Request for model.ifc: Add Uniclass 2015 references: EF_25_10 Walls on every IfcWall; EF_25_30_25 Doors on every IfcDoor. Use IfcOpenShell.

First a look at what the model holds.

```python
import ifcopenshell

model = ifcopenshell.open("model.ifc")
print(model.schema)
print("classifications:", [c.Name for c in model.by_type("IfcClassification")])
for ifc_class in ("IfcDoor", "IfcRoof", "IfcStair", "IfcWall", "IfcWindow"):
    print(ifc_class, len(model.by_type(ifc_class)))
```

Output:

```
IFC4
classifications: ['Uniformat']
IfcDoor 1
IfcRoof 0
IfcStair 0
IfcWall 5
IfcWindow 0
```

```python
import ifcopenshell
import ifcopenshell.api.classification

model = ifcopenshell.open("model.ifc")

system = ifcopenshell.api.classification.add_classification(model, classification="Uniclass 2015")

codes = {
    "IfcWall": ("EF_25_10", "Walls"),
    "IfcDoor": ("EF_25_30_25", "Doors"),
}
for ifc_class, (code, name) in codes.items():
    products = model.by_type(ifc_class)
    ifcopenshell.api.classification.add_reference(
        model, products=products, classification=system, identification=code, name=name
    )
    print(code, len(products))

model.write("model_rev.ifc")
```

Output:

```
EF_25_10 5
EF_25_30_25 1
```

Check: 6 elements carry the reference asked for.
